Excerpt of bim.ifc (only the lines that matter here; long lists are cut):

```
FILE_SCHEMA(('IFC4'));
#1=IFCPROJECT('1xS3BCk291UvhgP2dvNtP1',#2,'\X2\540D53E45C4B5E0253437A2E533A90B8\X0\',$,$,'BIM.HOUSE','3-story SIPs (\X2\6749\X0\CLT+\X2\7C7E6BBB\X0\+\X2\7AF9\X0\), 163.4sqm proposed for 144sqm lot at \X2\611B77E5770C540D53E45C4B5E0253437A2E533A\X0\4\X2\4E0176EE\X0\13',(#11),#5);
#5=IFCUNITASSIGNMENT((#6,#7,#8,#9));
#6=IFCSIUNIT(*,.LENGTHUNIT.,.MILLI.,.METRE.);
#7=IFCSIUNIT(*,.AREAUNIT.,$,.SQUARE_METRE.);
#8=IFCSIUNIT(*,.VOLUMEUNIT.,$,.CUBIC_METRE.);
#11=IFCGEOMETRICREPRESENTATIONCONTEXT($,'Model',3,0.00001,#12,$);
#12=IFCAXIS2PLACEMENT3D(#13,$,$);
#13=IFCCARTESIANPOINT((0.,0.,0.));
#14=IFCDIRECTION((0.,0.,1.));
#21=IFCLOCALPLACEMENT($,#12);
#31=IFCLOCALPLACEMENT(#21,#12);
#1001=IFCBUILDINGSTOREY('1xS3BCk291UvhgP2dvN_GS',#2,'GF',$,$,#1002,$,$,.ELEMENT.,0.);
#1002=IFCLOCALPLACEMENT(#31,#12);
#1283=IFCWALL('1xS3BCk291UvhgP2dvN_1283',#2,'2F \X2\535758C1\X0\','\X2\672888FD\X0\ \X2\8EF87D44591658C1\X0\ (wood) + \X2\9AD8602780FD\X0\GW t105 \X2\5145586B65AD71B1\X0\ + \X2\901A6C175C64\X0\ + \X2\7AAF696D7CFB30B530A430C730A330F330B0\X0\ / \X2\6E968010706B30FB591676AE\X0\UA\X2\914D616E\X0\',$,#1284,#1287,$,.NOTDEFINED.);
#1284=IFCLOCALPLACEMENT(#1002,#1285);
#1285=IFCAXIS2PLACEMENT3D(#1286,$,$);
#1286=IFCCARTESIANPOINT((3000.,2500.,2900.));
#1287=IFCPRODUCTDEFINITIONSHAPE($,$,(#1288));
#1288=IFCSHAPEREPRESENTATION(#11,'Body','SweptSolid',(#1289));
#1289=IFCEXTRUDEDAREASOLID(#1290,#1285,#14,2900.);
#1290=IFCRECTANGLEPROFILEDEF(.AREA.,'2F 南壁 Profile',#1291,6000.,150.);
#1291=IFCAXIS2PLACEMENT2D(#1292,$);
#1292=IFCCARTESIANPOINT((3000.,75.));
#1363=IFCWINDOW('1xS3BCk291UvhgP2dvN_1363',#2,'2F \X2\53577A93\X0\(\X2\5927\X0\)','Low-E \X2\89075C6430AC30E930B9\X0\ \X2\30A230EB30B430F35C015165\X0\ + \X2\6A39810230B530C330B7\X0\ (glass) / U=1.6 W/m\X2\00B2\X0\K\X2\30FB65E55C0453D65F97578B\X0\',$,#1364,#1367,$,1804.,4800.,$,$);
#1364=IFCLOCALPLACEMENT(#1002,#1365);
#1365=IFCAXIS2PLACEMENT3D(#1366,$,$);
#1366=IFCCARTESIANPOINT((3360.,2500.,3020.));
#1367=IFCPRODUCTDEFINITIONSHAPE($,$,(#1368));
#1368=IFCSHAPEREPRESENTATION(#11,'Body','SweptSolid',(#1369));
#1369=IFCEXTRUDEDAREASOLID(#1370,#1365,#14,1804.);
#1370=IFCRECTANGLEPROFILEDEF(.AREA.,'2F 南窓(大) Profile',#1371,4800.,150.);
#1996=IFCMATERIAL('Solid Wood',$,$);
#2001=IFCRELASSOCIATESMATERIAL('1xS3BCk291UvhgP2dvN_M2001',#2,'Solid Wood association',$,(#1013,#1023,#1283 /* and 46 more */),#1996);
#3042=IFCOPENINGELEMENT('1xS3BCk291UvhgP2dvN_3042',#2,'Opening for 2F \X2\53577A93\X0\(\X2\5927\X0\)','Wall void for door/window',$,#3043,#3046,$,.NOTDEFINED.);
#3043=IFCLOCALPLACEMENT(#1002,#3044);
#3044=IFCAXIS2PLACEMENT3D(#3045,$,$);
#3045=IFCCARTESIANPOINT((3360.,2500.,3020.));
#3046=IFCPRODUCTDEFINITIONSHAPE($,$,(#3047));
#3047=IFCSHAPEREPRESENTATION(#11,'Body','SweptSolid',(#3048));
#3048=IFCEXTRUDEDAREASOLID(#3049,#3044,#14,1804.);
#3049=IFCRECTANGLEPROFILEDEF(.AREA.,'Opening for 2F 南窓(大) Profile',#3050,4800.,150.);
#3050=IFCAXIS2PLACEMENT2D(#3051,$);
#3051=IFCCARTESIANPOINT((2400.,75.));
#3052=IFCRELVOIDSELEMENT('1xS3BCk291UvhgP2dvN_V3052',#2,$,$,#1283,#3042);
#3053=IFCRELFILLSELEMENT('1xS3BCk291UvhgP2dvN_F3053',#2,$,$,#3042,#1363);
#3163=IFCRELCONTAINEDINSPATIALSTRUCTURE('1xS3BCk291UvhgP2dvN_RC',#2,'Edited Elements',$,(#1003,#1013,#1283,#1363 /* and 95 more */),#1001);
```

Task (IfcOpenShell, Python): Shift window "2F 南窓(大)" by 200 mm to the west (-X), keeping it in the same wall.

```python
import ifcopenshell
import ifcopenshell.api.geometry
import ifcopenshell.util.placement
import ifcopenshell.util.unit

model = ifcopenshell.open("bim.ifc")
unit_scale = ifcopenshell.util.unit.calculate_unit_scale(model)

window = model.by_guid("1xS3BCk291UvhgP2dvN_1363")
opening = window.FillsVoids[0].RelatingOpeningElement
wall = opening.VoidsElements[0].RelatingBuildingElement

wall_matrix = ifcopenshell.util.placement.get_local_placement(wall.ObjectPlacement)
shift = wall_matrix[:3, 0] * -0.2 / unit_scale
before = ifcopenshell.util.placement.get_local_placement(window.ObjectPlacement)[:3, 3].copy()

# The window is not placed relative to its opening, so move both.
for product in (opening, window):
    matrix = ifcopenshell.util.placement.get_local_placement(product.ObjectPlacement)
    matrix[:3, 3] += shift
    ifcopenshell.api.geometry.edit_object_placement(model, product=product, matrix=matrix, is_si=False)

after = ifcopenshell.util.placement.get_local_placement(window.ObjectPlacement)[:3, 3]
print("window moved by", (after - before).round(3) + 0.0)

model.write("bim_rev.ifc")
```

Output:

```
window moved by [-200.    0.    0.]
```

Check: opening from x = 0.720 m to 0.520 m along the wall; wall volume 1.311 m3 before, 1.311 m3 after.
